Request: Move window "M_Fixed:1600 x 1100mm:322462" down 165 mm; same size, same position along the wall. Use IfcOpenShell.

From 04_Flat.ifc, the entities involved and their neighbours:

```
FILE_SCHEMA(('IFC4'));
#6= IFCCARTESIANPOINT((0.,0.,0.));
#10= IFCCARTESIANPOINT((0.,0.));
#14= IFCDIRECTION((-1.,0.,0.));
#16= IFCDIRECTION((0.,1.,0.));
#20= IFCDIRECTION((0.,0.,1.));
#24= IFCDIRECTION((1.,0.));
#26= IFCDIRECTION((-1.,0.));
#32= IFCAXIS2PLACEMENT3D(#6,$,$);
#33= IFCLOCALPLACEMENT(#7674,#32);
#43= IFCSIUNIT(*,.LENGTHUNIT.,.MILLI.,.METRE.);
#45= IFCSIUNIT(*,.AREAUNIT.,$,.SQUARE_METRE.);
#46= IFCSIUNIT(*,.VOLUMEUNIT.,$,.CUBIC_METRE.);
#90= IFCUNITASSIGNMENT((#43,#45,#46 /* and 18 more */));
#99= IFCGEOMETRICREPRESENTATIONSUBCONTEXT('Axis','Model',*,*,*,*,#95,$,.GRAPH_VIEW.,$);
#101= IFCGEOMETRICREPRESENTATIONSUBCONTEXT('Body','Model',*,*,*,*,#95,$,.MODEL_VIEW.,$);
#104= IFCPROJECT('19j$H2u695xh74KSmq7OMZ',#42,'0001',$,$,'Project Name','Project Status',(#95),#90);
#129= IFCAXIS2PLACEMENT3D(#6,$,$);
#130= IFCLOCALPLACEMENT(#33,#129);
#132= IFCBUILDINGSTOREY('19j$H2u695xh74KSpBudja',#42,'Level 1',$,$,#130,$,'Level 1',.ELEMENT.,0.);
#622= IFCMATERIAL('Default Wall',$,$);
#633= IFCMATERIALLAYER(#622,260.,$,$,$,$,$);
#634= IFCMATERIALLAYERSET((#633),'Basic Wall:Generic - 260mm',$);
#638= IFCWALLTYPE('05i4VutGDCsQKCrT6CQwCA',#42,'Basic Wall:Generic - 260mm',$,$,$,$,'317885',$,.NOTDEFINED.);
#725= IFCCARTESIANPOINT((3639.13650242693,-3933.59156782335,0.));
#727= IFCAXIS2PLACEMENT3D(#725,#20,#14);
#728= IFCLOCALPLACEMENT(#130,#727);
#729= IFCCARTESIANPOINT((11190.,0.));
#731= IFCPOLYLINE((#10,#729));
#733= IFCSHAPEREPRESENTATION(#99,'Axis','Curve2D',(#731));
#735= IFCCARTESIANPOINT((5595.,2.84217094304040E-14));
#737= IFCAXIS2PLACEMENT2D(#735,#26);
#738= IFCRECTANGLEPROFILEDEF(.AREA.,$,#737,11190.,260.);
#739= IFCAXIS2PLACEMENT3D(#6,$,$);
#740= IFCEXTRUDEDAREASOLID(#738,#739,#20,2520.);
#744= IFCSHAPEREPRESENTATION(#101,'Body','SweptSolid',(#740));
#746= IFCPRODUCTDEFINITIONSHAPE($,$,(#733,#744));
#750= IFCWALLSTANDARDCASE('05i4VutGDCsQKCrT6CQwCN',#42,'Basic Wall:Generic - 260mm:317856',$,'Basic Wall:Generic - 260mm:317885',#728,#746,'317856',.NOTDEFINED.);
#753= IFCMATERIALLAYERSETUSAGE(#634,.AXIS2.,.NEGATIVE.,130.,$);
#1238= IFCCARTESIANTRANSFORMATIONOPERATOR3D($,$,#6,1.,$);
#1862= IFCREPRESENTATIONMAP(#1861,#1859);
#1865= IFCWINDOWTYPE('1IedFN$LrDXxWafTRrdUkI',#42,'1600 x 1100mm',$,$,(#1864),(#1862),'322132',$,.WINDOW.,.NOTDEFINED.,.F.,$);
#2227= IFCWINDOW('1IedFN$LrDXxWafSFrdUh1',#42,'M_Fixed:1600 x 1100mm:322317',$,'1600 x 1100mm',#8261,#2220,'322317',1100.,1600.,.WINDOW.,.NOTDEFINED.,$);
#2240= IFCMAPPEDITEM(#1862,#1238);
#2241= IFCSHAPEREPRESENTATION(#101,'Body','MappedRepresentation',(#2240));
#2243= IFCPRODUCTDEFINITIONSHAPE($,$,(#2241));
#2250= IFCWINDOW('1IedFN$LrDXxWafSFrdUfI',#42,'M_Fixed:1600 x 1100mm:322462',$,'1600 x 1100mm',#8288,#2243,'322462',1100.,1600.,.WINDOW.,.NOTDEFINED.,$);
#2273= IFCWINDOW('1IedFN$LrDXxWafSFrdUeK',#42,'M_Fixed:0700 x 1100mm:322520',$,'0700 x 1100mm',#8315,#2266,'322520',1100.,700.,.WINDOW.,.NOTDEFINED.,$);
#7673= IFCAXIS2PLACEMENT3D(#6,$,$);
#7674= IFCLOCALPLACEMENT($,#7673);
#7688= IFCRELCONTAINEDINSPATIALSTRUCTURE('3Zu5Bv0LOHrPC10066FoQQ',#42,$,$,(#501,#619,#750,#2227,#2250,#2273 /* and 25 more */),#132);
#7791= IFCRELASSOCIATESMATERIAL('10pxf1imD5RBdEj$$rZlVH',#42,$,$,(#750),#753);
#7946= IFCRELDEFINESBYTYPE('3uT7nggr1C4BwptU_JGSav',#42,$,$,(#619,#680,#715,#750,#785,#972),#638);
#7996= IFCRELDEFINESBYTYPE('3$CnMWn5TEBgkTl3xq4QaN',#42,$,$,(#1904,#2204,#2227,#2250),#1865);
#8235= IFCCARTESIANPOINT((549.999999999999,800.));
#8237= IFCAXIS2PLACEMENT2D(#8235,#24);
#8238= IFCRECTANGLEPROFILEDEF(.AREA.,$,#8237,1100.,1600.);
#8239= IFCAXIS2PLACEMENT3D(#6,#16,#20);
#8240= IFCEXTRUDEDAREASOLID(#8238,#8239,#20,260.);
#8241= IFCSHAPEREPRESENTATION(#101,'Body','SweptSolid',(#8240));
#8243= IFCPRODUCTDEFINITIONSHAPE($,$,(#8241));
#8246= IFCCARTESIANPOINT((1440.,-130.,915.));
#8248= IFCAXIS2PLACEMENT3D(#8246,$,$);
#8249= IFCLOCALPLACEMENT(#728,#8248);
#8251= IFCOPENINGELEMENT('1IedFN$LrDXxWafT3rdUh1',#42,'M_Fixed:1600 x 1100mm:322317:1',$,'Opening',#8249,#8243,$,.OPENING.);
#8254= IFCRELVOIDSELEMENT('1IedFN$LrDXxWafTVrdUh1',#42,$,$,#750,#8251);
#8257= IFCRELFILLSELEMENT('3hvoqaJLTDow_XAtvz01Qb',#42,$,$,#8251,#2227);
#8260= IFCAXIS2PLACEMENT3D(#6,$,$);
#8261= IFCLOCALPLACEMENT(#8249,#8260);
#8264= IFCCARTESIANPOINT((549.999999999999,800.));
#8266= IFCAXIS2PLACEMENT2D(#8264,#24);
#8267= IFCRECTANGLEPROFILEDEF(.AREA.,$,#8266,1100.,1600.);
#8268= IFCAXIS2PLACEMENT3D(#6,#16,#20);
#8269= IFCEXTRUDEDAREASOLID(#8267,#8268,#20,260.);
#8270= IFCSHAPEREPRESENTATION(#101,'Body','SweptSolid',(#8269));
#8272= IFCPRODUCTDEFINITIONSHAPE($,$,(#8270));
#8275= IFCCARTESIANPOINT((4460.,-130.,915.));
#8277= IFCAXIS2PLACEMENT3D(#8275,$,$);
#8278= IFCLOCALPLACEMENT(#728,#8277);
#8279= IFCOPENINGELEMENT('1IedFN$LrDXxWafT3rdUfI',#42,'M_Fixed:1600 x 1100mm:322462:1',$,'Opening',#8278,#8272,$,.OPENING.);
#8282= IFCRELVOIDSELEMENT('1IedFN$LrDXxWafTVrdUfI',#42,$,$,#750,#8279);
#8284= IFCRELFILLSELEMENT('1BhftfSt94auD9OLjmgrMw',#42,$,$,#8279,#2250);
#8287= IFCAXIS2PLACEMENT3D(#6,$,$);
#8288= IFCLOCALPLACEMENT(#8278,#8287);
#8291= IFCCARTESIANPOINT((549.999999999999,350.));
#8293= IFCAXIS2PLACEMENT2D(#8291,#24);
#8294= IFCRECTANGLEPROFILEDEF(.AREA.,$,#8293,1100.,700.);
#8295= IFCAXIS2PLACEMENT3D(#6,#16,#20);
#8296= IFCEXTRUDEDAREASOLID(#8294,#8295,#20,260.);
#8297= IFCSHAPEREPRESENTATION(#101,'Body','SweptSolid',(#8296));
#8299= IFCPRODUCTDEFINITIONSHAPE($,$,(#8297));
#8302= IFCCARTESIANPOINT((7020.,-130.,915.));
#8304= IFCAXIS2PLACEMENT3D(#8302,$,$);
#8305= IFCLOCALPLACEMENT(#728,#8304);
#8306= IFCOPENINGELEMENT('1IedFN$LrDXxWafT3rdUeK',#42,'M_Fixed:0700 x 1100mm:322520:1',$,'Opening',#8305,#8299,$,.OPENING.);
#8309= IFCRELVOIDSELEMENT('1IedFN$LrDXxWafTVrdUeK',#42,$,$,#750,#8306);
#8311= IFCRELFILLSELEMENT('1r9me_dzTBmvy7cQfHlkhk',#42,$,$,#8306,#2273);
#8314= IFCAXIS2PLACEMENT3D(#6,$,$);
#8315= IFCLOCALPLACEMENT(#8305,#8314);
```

```python
import numpy as np
import ifcopenshell
import ifcopenshell.api.geometry
import ifcopenshell.util.placement
import ifcopenshell.util.unit

model = ifcopenshell.open("04_Flat.ifc")
unit_scale = ifcopenshell.util.unit.calculate_unit_scale(model)

window = model.by_id(2250)
opening = window.FillsVoids[0].RelatingOpeningElement
dz = -0.165 / unit_scale

shift = np.array([0.0, 0.0, dz])
# The window is placed relative to its opening, so it follows when the opening moves.
matrix = ifcopenshell.util.placement.get_local_placement(opening.ObjectPlacement)
matrix[:3, 3] += shift
ifcopenshell.api.geometry.edit_object_placement(
    model, product=opening, matrix=matrix, is_si=False, should_transform_children=True
)

print(f"moved by {dz * unit_scale:+.3f} m")

model.write("04_Flat_updated.ifc")
```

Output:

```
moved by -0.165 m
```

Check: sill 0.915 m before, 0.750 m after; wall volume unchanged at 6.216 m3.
